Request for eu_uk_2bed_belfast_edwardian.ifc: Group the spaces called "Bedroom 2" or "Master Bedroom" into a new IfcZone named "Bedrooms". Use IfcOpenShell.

First a look at what the model holds.

```python
import ifcopenshell

model = ifcopenshell.open("eu_uk_2bed_belfast_edwardian.ifc")
print(model.schema)
seen = {}
for space in model.by_type("IfcSpace"):
    seen[space.LongName] = seen.get(space.LongName, 0) + 1
for name, count in sorted(seen.items(), key=str):
    print(count, "x", name)
print("zones:", [z.Name for z in model.by_type("IfcZone")][:20])
```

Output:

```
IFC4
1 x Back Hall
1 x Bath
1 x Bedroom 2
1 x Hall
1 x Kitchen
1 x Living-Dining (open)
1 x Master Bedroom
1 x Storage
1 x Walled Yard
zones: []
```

```python
import ifcopenshell
import ifcopenshell.api.group
import ifcopenshell.api.root

model = ifcopenshell.open("eu_uk_2bed_belfast_edwardian.ifc")

names = {"Bedroom 2", "Master Bedroom"}
spaces = [s for s in model.by_type("IfcSpace") if s.LongName in names]

zone = ifcopenshell.api.root.create_entity(model, ifc_class="IfcZone", name="Bedrooms")
ifcopenshell.api.group.assign_group(model, products=spaces, group=zone)
print(len(spaces), "spaces in", zone.Name)

model.write("eu_uk_2bed_belfast_edwardian_edited.ifc")
```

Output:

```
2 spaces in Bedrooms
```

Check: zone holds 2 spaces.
